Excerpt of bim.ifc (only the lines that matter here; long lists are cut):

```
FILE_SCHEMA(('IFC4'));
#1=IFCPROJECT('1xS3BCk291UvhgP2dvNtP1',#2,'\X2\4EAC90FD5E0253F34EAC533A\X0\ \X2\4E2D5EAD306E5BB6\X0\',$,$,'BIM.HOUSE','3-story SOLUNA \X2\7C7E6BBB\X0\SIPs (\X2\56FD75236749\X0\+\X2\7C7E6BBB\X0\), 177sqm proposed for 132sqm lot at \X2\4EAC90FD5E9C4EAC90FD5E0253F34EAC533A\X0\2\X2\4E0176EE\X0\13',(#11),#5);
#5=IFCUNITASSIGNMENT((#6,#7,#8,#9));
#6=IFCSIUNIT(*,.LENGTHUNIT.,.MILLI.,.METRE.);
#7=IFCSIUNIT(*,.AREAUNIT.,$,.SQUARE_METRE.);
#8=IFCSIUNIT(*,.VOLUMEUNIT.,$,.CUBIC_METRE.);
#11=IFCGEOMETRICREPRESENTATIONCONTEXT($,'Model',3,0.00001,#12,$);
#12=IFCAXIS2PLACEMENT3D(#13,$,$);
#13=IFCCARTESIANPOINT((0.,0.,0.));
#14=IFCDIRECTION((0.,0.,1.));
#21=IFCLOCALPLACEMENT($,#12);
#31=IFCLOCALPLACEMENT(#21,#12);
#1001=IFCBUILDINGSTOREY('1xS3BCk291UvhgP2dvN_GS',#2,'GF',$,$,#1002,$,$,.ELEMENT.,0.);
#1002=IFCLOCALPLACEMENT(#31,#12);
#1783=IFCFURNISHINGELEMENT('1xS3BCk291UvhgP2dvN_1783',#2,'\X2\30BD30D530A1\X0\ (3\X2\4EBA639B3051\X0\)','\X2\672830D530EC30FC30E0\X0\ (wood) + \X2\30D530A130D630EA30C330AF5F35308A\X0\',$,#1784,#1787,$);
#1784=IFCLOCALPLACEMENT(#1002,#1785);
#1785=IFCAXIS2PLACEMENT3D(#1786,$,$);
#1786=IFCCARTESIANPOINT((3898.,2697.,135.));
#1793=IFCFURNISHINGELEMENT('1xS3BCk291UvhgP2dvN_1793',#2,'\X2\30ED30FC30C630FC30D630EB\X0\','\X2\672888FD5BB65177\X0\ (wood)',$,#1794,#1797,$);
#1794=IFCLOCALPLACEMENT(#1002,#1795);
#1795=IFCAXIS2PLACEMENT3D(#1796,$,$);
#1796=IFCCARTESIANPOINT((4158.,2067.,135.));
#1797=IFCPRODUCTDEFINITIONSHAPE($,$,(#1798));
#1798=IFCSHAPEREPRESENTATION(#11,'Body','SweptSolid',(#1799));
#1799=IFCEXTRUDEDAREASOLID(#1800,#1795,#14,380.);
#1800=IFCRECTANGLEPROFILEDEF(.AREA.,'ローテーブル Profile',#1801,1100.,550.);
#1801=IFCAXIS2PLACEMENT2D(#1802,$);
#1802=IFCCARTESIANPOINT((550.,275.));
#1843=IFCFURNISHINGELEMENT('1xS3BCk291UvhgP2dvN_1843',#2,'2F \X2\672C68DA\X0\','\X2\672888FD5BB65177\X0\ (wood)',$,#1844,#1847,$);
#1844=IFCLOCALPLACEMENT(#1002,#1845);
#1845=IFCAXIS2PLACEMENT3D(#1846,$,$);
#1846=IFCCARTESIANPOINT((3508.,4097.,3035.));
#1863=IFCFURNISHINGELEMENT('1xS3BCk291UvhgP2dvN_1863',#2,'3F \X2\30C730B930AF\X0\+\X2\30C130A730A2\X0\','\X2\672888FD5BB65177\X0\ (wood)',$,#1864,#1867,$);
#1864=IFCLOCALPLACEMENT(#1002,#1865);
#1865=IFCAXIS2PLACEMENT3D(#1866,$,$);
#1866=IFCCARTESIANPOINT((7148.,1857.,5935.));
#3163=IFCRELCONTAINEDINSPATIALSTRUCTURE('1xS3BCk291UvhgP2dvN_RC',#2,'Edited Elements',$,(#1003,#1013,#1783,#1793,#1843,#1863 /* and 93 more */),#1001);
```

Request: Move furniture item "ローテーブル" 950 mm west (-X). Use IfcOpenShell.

```python
import ifcopenshell
import ifcopenshell.api.geometry
import ifcopenshell.util.placement
import ifcopenshell.util.unit

model = ifcopenshell.open("bim.ifc")
unit_scale = ifcopenshell.util.unit.calculate_unit_scale(model)

item = model.by_guid("1xS3BCk291UvhgP2dvN_1793")
matrix = ifcopenshell.util.placement.get_local_placement(item.ObjectPlacement)
matrix[0, 3] -= 0.95 / unit_scale
ifcopenshell.api.geometry.edit_object_placement(model, product=item, matrix=matrix, is_si=False)

print(ifcopenshell.util.placement.get_local_placement(item.ObjectPlacement).round(3) + 0.0)

model.write("bim_edited.ifc")
```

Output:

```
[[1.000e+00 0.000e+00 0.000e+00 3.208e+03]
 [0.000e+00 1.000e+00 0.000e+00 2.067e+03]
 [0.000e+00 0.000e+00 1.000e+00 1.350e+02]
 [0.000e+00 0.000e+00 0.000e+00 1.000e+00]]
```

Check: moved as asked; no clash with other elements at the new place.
